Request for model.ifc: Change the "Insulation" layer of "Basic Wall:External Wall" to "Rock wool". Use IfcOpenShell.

First a look at what the model holds.

```python
import ifcopenshell
import ifcopenshell.util.element

model = ifcopenshell.open("model.ifc")
print(model.schema)
for layer_set in model.by_type("IfcMaterialLayerSet"):
    if layer_set.LayerSetName == "Basic Wall:External Wall":
        for layer in layer_set.MaterialLayers:
            print(layer.id(), layer.Material and layer.Material.Name, layer.LayerThickness, sep=" | ")
        print(len(ifcopenshell.util.element.get_elements_by_material(model, layer_set)), "elements and types use it")
print(sorted(m.Name for m in model.by_type("IfcMaterial") if m.Name)[:60])
```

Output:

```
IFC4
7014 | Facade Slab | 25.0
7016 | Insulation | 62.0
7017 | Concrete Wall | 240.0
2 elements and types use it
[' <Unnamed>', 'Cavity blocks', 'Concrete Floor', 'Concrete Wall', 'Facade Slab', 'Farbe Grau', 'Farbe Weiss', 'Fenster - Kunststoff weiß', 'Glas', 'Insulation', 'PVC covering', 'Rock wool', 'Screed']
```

```python
import ifcopenshell
import ifcopenshell.api.material

model = ifcopenshell.open("model.ifc")

layer_set = next(s for s in model.by_type("IfcMaterialLayerSet") if s.LayerSetName == "Basic Wall:External Wall")
layer = next(l for l in layer_set.MaterialLayers if l.Material and l.Material.Name == "Insulation")
material = next(m for m in model.by_type("IfcMaterial") if m.Name == "Rock wool")

# Point this one layer at the other material; renaming the old one would change it everywhere.
ifcopenshell.api.material.edit_layer(model, layer=layer, attributes={}, material=material)

print([l.Material.Name if l.Material else None for l in layer_set.MaterialLayers])

model.write("model-out.ifc")
```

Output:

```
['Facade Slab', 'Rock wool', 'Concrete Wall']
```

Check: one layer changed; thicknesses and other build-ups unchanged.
